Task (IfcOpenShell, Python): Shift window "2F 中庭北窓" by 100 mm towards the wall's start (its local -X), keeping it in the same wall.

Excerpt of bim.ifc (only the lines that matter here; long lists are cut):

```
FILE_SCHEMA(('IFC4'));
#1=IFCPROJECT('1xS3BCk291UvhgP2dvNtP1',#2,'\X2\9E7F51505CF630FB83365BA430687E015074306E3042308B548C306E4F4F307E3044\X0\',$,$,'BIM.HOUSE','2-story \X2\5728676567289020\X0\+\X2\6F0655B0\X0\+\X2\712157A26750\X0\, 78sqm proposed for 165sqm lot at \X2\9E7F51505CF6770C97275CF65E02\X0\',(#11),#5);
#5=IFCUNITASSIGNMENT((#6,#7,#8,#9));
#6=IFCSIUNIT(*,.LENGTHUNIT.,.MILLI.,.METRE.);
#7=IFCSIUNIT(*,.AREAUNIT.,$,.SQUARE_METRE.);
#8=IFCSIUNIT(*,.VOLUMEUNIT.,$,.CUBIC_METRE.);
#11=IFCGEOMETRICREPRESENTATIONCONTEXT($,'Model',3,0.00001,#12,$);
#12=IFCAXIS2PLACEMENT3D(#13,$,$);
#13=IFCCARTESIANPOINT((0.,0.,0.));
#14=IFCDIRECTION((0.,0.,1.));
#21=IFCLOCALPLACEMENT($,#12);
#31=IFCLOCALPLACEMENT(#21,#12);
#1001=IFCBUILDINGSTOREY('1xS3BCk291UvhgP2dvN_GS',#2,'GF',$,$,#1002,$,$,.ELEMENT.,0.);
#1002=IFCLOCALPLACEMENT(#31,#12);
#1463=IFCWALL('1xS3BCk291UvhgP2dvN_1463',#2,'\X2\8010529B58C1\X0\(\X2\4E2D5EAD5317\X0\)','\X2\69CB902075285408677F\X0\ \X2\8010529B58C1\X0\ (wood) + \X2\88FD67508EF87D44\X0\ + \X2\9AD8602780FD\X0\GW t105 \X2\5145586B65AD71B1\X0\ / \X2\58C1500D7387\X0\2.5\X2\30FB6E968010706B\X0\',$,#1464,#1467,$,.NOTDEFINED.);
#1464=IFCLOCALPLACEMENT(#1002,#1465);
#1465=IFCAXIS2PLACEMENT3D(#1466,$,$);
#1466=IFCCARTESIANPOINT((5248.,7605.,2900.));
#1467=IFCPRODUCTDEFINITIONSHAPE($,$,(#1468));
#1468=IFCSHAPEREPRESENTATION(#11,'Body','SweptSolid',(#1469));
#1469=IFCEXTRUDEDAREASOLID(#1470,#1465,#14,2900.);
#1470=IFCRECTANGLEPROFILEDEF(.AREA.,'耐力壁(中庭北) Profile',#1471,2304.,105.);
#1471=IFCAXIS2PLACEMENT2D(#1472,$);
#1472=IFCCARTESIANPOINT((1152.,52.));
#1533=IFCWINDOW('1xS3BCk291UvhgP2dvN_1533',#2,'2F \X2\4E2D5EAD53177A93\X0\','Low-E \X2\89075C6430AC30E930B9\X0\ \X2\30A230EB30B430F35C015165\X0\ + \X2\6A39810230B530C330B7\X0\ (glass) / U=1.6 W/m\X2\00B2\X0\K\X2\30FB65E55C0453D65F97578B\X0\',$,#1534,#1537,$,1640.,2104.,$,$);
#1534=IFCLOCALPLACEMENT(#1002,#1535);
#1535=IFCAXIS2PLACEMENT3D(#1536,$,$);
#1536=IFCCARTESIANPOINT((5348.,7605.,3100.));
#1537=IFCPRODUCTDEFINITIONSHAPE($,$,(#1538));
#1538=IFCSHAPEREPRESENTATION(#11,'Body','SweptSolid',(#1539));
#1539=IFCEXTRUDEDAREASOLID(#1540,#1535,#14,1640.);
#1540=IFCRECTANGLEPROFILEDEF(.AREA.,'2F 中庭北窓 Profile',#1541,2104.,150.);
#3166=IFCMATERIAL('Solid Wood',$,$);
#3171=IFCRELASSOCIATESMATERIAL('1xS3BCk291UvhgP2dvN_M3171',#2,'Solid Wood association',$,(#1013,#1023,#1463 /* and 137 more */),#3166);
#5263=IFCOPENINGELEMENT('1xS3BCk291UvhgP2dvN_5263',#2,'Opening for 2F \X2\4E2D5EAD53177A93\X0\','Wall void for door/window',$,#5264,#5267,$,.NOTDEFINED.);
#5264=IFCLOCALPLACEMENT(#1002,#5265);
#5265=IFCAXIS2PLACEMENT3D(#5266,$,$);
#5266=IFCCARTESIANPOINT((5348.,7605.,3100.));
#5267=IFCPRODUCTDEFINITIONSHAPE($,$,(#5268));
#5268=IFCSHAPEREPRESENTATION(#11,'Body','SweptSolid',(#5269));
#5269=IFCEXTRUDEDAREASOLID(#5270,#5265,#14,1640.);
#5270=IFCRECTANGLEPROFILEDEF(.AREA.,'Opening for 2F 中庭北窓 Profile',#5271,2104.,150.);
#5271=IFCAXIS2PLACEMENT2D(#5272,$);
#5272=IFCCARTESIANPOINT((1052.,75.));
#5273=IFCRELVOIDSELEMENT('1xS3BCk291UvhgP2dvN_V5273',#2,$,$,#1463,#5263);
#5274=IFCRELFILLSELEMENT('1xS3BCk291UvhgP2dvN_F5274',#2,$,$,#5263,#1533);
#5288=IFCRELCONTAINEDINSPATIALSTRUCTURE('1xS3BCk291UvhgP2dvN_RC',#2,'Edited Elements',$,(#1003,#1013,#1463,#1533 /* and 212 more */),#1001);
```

```python
import ifcopenshell
import ifcopenshell.api.geometry
import ifcopenshell.util.placement
import ifcopenshell.util.unit

model = ifcopenshell.open("bim.ifc")
unit_scale = ifcopenshell.util.unit.calculate_unit_scale(model)

window = model.by_id(1533)
opening = window.FillsVoids[0].RelatingOpeningElement
wall = opening.VoidsElements[0].RelatingBuildingElement

wall_matrix = ifcopenshell.util.placement.get_local_placement(wall.ObjectPlacement)
shift = wall_matrix[:3, 0] * -0.1 / unit_scale
before = ifcopenshell.util.placement.get_local_placement(window.ObjectPlacement)[:3, 3].copy()

# The window is not placed relative to its opening, so move both.
for product in (opening, window):
    matrix = ifcopenshell.util.placement.get_local_placement(product.ObjectPlacement)
    matrix[:3, 3] += shift
    ifcopenshell.api.geometry.edit_object_placement(model, product=product, matrix=matrix, is_si=False)

after = ifcopenshell.util.placement.get_local_placement(window.ObjectPlacement)[:3, 3]
print("window moved by", (after - before).round(3) + 0.0)

model.write("bim-out.ifc")
```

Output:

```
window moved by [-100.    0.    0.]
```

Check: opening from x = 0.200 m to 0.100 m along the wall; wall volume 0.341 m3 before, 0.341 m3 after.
